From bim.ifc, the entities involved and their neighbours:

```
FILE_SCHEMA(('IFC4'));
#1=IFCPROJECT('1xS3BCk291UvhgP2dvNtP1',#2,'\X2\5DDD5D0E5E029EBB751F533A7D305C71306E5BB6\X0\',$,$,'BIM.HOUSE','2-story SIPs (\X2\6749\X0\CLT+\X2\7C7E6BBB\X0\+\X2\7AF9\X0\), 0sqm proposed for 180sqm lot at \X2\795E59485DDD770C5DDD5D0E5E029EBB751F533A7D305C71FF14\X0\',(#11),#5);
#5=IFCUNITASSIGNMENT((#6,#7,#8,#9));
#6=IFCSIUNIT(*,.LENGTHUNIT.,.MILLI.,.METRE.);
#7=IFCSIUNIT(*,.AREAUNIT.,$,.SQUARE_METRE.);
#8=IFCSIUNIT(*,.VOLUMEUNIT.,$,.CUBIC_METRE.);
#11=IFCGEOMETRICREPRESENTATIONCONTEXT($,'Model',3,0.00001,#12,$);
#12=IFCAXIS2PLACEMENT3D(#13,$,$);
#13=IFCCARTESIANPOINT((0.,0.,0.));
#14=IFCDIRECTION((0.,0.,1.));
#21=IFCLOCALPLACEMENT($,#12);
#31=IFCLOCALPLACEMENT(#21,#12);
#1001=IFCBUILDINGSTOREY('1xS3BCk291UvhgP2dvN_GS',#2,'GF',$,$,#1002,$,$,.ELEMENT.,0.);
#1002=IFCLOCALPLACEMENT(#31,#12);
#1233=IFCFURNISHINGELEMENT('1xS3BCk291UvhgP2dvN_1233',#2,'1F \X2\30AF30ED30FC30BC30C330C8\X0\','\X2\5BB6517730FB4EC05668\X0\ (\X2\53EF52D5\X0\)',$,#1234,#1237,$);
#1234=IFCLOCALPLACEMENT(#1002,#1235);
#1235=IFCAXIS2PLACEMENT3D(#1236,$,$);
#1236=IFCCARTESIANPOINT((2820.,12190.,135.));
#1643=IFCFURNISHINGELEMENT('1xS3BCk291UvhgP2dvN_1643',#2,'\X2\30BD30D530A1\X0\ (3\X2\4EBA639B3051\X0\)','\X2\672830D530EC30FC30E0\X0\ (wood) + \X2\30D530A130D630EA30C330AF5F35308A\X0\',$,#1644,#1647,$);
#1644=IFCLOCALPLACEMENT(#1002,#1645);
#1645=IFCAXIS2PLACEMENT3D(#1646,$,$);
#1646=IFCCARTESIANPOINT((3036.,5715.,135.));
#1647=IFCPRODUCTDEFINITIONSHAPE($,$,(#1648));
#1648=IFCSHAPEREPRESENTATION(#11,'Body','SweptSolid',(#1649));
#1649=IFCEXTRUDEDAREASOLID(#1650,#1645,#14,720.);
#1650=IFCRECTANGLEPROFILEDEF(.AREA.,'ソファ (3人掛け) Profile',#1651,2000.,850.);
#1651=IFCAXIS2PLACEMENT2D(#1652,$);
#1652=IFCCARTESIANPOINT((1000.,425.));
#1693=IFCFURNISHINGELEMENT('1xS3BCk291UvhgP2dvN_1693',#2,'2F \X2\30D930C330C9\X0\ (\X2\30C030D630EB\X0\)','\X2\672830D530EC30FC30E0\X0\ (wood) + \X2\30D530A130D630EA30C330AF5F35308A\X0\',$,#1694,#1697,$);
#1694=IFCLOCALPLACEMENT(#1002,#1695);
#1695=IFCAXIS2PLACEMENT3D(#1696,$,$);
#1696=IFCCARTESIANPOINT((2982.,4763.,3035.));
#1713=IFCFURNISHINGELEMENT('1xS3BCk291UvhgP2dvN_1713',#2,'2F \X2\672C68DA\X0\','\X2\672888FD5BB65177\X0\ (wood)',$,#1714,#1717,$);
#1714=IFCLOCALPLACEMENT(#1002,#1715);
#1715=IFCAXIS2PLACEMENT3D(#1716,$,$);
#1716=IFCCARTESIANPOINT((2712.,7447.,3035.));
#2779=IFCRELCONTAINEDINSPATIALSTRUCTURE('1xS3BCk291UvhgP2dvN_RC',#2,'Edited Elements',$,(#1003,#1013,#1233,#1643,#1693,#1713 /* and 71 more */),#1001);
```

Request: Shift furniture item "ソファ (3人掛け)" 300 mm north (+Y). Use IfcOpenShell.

```python
import ifcopenshell
import ifcopenshell.api.geometry
import ifcopenshell.util.placement

model = ifcopenshell.open("bim.ifc")

item = model.by_guid("1xS3BCk291UvhgP2dvN_1643")
matrix = ifcopenshell.util.placement.get_local_placement(item.ObjectPlacement)
matrix[1, 3] += 300.0
ifcopenshell.api.geometry.edit_object_placement(model, product=item, matrix=matrix, is_si=False)

print(ifcopenshell.util.placement.get_local_placement(item.ObjectPlacement).round(3) + 0.0)

model.write("bim_updated.ifc")
```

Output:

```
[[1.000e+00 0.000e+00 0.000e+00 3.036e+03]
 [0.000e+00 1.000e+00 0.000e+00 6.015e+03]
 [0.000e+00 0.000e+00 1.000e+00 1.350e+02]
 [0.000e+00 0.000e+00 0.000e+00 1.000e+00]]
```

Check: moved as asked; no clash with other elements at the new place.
